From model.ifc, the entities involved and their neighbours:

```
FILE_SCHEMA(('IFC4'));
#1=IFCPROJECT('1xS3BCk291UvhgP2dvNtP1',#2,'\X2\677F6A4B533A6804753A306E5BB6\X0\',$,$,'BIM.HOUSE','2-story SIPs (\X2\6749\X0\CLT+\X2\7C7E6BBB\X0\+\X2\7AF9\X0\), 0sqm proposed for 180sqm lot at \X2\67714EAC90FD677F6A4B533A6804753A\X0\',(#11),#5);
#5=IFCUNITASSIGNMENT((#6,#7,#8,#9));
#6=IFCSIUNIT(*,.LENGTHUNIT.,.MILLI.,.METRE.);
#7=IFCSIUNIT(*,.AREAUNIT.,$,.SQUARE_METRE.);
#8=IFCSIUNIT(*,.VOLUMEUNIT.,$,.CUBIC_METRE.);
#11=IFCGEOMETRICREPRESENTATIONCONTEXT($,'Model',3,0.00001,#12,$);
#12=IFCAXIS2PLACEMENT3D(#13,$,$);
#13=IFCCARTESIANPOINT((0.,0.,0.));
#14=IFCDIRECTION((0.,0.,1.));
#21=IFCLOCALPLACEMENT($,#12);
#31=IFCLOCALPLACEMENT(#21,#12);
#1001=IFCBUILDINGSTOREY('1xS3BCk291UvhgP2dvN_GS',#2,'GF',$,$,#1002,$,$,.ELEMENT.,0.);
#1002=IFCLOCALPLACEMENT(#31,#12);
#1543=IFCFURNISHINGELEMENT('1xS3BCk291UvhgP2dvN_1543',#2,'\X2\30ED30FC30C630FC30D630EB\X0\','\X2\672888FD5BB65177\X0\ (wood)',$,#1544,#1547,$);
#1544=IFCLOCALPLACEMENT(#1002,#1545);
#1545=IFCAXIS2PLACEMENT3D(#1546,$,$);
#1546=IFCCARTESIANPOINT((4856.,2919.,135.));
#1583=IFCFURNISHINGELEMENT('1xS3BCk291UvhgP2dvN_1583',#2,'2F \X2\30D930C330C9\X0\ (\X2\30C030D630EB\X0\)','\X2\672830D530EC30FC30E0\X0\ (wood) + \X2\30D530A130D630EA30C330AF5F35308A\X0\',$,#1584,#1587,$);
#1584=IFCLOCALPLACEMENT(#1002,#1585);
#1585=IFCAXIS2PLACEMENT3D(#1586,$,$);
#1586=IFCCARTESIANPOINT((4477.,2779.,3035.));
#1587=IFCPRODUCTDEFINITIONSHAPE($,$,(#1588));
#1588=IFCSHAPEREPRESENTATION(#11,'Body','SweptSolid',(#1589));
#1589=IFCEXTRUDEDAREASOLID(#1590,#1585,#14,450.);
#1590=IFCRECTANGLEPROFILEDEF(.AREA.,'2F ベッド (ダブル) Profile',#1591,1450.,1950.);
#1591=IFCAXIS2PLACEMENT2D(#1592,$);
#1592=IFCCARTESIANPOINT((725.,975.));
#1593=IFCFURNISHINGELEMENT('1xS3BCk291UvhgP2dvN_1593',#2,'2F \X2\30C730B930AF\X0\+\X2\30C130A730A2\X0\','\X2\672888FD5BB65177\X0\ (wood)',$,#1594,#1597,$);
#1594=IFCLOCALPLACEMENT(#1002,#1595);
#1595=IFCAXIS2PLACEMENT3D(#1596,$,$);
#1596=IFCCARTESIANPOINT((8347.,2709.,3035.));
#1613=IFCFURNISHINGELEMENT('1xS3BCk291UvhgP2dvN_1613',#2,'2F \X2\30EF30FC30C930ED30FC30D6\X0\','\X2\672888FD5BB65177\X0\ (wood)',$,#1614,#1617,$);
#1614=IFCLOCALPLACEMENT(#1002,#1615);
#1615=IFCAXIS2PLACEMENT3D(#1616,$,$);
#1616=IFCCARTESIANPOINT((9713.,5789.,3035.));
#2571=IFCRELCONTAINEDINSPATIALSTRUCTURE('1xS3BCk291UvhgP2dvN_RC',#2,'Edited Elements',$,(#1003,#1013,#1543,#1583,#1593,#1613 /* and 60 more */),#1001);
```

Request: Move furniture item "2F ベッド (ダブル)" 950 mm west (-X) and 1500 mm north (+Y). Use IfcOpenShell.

```python
import ifcopenshell
import ifcopenshell.api.geometry
import ifcopenshell.util.placement
import ifcopenshell.util.unit

model = ifcopenshell.open("model.ifc")
unit_scale = ifcopenshell.util.unit.calculate_unit_scale(model)

item = model.by_guid("1xS3BCk291UvhgP2dvN_1583")
matrix = ifcopenshell.util.placement.get_local_placement(item.ObjectPlacement)
matrix[0, 3] -= 0.95 / unit_scale
matrix[1, 3] += 1.5 / unit_scale
ifcopenshell.api.geometry.edit_object_placement(model, product=item, matrix=matrix, is_si=False)

print(ifcopenshell.util.placement.get_local_placement(item.ObjectPlacement).round(3) + 0.0)

model.write("model_edited.ifc")
```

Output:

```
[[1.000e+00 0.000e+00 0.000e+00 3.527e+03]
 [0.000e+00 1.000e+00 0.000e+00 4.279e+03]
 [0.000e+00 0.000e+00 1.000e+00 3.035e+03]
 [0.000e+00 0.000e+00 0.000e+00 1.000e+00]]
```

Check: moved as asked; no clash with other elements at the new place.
